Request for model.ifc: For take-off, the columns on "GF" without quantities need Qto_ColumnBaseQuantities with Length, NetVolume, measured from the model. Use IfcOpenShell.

First a look at what the model holds.

```python
import ifcopenshell
import ifcopenshell.util.element
import ifcopenshell.util.unit

model = ifcopenshell.open("model.ifc")
print(model.schema)
for unit_type in ("LENGTHUNIT", "AREAUNIT", "VOLUMEUNIT"):
    print(unit_type, ifcopenshell.util.unit.calculate_unit_scale(model, unit_type))
storey = next(s for s in model.by_type("IfcBuildingStorey") if s.Name == "GF")
columns = [e for e in ifcopenshell.util.element.get_decomposition(storey) if e.is_a("IfcColumn")]
for e in sorted(columns, key=lambda e: e.id()):
    print(e.id(), e.is_a(), e.Name, list(ifcopenshell.util.element.get_psets(e, qtos_only=True)), sep=" | ")
```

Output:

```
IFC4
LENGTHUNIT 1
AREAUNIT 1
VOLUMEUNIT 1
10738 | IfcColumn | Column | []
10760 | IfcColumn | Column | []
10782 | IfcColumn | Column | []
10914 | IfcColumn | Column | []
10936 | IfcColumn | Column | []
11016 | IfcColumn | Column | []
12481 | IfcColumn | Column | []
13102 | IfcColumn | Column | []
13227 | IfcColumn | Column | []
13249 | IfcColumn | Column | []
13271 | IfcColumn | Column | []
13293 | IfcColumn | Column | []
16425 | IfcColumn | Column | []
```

```python
import ifcopenshell
import ifcopenshell.api.pset
import ifcopenshell.geom
import ifcopenshell.util.element
import ifcopenshell.util.shape
import ifcopenshell.util.unit

model = ifcopenshell.open("model.ifc")
unit_scale = ifcopenshell.util.unit.calculate_unit_scale(model)
volume_scale = ifcopenshell.util.unit.calculate_unit_scale(model, "VOLUMEUNIT")
settings = ifcopenshell.geom.settings()

storey = next(s for s in model.by_type("IfcBuildingStorey") if s.Name == "GF")
columns = [e for e in ifcopenshell.util.element.get_decomposition(storey) if e.is_a("IfcColumn")]

for e in sorted(columns, key=lambda e: e.id()):
    if ifcopenshell.util.element.get_psets(e, qtos_only=True, should_inherit=False):
        continue
    # Geometry comes back in metres, in the element's own axes.
    shape = ifcopenshell.geom.create_shape(settings, e)
    values = {
        "Length": ifcopenshell.util.shape.get_z(shape.geometry) / unit_scale,
        "NetVolume": ifcopenshell.util.shape.get_volume(shape.geometry) / volume_scale,
    }
    qto = ifcopenshell.api.pset.add_qto(model, product=e, name="Qto_ColumnBaseQuantities")
    ifcopenshell.api.pset.edit_qto(model, qto=qto, properties=values)
    print(e.id(), {k: round(v, 3) for k, v in values.items()})

model.write("model-out.ifc")
```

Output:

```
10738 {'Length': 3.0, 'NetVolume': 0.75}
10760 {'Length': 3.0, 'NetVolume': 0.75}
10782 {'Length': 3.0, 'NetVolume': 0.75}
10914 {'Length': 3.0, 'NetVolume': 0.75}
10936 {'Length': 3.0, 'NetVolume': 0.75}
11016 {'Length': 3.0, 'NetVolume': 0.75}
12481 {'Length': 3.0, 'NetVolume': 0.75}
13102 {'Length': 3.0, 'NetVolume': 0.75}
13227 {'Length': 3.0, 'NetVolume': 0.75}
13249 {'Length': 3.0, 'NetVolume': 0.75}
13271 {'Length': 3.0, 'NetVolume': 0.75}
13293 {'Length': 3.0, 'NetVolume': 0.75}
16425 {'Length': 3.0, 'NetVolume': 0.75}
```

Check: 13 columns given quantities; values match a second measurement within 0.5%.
